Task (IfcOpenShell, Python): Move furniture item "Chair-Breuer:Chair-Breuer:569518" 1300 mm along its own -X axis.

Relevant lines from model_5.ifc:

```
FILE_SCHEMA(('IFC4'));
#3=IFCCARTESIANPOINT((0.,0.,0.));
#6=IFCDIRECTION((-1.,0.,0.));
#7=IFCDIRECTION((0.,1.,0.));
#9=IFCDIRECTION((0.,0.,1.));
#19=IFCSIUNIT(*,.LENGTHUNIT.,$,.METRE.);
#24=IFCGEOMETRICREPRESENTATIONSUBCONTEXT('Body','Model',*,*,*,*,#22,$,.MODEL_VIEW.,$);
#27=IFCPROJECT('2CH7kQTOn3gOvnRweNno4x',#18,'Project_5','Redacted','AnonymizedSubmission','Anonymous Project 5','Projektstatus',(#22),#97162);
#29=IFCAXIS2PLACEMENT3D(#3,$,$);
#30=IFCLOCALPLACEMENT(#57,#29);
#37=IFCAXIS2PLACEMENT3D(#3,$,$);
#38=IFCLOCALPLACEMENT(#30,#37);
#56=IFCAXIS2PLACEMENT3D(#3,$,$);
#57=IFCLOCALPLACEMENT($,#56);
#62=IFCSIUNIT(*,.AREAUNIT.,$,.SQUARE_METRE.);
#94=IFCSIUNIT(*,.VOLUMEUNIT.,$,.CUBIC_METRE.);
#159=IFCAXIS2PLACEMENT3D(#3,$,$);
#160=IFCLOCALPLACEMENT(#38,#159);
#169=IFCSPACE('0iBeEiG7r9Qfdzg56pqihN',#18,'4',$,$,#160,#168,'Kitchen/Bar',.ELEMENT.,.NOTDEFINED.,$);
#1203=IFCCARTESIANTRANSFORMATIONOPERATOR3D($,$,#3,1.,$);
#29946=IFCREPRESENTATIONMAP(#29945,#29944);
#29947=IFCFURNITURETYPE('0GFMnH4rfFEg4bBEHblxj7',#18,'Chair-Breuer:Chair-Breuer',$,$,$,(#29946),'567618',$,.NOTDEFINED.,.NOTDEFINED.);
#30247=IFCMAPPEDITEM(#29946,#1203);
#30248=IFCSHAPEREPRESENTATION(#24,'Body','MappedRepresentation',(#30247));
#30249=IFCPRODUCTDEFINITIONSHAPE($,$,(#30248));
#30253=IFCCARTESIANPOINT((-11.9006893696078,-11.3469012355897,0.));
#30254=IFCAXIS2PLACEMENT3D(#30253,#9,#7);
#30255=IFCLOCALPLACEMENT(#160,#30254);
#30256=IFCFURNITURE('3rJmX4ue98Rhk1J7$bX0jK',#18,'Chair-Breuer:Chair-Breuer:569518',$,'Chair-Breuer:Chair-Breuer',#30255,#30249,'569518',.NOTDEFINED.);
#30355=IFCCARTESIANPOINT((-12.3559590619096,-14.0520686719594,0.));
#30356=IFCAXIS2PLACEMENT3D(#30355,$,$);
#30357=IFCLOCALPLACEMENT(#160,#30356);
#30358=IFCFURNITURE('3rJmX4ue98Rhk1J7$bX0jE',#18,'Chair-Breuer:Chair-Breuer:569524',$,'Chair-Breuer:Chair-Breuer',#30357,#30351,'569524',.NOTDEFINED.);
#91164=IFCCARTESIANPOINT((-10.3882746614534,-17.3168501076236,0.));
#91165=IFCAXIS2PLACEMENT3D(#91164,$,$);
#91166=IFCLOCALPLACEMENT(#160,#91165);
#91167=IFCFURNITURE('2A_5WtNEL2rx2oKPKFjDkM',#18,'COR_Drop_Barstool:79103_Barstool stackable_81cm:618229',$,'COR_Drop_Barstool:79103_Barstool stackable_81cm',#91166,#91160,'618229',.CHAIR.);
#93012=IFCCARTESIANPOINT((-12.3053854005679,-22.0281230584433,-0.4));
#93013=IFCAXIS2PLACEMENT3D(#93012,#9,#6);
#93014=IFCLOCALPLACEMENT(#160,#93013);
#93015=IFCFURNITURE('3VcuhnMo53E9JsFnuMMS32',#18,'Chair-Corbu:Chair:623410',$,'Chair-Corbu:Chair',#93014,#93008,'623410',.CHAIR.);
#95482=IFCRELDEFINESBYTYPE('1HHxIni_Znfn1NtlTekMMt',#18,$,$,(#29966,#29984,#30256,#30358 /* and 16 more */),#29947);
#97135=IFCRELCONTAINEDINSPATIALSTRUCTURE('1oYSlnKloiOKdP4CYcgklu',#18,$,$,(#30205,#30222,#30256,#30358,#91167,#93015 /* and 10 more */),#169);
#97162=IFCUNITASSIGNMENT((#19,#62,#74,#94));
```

```python
import ifcopenshell
import ifcopenshell.api.geometry
import ifcopenshell.util.placement
import ifcopenshell.util.unit

model = ifcopenshell.open("model_5.ifc")
unit_scale = ifcopenshell.util.unit.calculate_unit_scale(model)

item = model.by_guid("3rJmX4ue98Rhk1J7$bX0jK")
matrix = ifcopenshell.util.placement.get_local_placement(item.ObjectPlacement)
matrix[:3, 3] -= matrix[:3, 0] * 1.3 / unit_scale
ifcopenshell.api.geometry.edit_object_placement(model, product=item, matrix=matrix, is_si=False)

print(ifcopenshell.util.placement.get_local_placement(item.ObjectPlacement).round(3) + 0.0)

model.write("model_5_updated.ifc")
```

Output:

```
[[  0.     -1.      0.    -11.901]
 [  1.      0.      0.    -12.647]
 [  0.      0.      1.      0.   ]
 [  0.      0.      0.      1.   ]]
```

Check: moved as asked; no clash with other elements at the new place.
